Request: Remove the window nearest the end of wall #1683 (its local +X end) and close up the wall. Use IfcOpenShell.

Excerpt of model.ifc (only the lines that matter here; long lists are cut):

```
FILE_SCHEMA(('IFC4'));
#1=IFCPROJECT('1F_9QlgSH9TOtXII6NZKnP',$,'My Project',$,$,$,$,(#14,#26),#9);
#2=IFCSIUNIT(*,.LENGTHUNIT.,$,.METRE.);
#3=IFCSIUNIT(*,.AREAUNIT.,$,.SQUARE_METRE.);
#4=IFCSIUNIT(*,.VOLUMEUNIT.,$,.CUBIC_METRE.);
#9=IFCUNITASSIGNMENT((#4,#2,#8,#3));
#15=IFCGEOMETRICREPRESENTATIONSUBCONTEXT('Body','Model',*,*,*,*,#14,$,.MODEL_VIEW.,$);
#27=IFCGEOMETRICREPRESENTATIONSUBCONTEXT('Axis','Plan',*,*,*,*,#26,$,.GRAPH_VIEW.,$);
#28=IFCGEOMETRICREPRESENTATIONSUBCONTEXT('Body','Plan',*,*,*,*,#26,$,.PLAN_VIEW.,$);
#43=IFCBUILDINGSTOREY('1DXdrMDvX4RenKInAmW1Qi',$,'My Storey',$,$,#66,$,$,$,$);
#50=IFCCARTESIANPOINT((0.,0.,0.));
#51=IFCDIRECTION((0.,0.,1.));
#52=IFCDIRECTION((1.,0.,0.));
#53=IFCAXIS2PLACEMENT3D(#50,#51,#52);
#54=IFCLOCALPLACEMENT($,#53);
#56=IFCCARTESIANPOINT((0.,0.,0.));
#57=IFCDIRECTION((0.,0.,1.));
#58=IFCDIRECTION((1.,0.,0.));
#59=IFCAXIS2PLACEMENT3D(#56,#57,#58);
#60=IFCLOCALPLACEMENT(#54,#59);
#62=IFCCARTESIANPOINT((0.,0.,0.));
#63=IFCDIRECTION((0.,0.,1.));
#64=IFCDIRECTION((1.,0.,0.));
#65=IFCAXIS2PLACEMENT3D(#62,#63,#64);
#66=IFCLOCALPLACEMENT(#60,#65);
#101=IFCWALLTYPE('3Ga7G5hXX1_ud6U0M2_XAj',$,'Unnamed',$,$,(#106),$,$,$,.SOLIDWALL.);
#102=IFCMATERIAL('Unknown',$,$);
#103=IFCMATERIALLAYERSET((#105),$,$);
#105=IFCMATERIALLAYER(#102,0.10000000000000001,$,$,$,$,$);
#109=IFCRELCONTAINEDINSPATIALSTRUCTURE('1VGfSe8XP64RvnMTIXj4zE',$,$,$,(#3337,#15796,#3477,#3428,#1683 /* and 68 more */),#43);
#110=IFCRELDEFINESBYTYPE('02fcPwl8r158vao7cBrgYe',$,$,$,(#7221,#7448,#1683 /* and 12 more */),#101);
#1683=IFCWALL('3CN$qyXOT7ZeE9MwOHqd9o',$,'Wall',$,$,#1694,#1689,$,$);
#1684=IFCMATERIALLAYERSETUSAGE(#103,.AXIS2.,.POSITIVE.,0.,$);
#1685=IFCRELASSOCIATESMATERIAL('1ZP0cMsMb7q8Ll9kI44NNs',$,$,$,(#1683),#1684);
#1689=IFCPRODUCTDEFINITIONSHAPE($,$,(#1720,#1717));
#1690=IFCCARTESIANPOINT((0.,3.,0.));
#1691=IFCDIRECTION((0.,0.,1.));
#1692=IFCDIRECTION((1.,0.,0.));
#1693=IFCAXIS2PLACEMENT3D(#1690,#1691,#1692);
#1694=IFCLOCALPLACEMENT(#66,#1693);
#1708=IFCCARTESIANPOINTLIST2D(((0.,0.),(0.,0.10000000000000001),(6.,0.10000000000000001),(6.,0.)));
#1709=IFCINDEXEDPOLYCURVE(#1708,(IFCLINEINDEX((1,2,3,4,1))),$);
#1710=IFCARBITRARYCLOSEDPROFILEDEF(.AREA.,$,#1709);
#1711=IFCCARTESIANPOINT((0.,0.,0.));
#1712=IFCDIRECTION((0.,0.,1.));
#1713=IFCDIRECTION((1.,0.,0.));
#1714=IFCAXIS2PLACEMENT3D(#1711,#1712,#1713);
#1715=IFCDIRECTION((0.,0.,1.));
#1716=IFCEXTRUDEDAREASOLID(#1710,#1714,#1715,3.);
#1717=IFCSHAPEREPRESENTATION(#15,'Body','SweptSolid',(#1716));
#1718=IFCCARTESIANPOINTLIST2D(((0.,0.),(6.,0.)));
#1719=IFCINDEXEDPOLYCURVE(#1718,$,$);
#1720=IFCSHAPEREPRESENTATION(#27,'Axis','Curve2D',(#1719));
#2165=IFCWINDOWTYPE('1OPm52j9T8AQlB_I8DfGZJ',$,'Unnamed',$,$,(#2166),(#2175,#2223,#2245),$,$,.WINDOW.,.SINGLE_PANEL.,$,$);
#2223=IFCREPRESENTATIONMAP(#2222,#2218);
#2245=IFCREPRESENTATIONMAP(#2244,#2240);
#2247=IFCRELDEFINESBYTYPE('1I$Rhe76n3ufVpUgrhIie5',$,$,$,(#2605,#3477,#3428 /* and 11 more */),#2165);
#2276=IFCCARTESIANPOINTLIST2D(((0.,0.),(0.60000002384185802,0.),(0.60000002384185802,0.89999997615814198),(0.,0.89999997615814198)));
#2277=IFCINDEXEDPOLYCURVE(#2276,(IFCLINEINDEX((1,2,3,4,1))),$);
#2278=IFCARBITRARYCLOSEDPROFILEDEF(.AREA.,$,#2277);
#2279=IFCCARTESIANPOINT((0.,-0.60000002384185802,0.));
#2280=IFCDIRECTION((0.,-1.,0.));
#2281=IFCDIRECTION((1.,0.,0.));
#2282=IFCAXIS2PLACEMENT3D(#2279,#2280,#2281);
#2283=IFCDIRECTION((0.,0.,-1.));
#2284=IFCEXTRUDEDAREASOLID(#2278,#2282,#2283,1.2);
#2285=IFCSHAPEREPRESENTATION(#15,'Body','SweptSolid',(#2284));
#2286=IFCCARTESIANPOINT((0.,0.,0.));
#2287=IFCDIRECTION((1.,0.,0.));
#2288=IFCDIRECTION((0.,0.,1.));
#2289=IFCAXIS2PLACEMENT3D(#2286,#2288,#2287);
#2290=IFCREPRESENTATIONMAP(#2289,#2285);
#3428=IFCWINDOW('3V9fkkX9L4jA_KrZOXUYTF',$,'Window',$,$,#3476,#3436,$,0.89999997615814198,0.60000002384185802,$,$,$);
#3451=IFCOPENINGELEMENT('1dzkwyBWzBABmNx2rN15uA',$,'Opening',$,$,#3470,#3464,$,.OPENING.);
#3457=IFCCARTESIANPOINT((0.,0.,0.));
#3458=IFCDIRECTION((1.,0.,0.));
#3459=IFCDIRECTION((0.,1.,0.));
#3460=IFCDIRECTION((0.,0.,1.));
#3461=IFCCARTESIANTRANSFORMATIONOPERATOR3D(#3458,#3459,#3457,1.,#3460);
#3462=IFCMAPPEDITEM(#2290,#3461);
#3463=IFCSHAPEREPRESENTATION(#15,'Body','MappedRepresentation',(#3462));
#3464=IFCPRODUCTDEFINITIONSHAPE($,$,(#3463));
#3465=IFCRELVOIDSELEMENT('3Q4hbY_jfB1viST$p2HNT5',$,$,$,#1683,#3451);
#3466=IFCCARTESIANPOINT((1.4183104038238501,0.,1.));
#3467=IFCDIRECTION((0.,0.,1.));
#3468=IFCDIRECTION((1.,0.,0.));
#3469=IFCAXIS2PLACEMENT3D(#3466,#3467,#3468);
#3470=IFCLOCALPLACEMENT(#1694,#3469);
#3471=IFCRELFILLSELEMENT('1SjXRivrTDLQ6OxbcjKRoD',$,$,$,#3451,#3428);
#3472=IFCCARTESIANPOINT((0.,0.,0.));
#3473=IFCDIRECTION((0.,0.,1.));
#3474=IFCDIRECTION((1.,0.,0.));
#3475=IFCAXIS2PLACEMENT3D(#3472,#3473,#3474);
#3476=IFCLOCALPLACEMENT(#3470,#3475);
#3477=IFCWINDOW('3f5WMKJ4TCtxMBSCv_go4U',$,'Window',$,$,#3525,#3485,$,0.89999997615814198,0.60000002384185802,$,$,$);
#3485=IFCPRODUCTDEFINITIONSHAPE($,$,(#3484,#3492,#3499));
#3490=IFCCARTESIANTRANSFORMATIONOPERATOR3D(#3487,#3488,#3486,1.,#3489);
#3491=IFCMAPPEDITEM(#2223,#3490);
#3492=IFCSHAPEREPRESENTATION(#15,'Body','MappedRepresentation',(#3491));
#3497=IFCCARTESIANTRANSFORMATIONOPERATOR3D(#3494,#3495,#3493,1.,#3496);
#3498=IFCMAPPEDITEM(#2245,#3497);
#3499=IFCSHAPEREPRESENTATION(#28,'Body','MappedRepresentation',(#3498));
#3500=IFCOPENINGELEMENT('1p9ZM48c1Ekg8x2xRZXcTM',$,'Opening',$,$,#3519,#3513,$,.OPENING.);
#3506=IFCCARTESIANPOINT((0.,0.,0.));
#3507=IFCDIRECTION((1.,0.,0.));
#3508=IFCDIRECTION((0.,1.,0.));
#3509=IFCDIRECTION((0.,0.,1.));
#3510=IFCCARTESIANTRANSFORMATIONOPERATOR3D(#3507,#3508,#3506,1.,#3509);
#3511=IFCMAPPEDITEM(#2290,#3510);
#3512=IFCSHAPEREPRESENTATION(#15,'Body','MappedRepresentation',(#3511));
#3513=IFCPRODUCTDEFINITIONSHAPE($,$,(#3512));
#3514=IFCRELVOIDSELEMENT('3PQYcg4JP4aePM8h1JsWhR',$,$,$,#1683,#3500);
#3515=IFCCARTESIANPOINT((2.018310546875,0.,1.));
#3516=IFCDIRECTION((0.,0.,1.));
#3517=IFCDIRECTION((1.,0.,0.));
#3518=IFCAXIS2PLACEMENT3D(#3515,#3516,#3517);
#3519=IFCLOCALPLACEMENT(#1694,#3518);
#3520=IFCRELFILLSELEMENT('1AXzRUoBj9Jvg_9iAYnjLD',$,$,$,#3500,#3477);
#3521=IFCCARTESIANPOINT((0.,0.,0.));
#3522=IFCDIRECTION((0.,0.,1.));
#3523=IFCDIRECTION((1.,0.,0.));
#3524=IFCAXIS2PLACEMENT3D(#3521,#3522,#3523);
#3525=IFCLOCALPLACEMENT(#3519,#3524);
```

```python
import ifcopenshell
import ifcopenshell.api.feature
import ifcopenshell.api.root
import ifcopenshell.geom
import ifcopenshell.util.shape

model = ifcopenshell.open("model.ifc")
settings = ifcopenshell.geom.settings()


def volume(element):
    """Net volume in cubic metres, openings subtracted."""
    shape = ifcopenshell.geom.create_shape(settings, element)
    return ifcopenshell.util.shape.get_volume(shape.geometry)


window = model.by_guid("3f5WMKJ4TCtxMBSCv_go4U")
opening = window.FillsVoids[0].RelatingOpeningElement
wall = opening.VoidsElements[0].RelatingBuildingElement
before = volume(wall)

ifcopenshell.api.root.remove_product(model, product=window)
ifcopenshell.api.feature.remove_feature(model, feature=opening)

after = volume(wall)

print(f"wall volume {before:.3f} -> {after:.3f} m3")

model.write("model_rev.ifc")
```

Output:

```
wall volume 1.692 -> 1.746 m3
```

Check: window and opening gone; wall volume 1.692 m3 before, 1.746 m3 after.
